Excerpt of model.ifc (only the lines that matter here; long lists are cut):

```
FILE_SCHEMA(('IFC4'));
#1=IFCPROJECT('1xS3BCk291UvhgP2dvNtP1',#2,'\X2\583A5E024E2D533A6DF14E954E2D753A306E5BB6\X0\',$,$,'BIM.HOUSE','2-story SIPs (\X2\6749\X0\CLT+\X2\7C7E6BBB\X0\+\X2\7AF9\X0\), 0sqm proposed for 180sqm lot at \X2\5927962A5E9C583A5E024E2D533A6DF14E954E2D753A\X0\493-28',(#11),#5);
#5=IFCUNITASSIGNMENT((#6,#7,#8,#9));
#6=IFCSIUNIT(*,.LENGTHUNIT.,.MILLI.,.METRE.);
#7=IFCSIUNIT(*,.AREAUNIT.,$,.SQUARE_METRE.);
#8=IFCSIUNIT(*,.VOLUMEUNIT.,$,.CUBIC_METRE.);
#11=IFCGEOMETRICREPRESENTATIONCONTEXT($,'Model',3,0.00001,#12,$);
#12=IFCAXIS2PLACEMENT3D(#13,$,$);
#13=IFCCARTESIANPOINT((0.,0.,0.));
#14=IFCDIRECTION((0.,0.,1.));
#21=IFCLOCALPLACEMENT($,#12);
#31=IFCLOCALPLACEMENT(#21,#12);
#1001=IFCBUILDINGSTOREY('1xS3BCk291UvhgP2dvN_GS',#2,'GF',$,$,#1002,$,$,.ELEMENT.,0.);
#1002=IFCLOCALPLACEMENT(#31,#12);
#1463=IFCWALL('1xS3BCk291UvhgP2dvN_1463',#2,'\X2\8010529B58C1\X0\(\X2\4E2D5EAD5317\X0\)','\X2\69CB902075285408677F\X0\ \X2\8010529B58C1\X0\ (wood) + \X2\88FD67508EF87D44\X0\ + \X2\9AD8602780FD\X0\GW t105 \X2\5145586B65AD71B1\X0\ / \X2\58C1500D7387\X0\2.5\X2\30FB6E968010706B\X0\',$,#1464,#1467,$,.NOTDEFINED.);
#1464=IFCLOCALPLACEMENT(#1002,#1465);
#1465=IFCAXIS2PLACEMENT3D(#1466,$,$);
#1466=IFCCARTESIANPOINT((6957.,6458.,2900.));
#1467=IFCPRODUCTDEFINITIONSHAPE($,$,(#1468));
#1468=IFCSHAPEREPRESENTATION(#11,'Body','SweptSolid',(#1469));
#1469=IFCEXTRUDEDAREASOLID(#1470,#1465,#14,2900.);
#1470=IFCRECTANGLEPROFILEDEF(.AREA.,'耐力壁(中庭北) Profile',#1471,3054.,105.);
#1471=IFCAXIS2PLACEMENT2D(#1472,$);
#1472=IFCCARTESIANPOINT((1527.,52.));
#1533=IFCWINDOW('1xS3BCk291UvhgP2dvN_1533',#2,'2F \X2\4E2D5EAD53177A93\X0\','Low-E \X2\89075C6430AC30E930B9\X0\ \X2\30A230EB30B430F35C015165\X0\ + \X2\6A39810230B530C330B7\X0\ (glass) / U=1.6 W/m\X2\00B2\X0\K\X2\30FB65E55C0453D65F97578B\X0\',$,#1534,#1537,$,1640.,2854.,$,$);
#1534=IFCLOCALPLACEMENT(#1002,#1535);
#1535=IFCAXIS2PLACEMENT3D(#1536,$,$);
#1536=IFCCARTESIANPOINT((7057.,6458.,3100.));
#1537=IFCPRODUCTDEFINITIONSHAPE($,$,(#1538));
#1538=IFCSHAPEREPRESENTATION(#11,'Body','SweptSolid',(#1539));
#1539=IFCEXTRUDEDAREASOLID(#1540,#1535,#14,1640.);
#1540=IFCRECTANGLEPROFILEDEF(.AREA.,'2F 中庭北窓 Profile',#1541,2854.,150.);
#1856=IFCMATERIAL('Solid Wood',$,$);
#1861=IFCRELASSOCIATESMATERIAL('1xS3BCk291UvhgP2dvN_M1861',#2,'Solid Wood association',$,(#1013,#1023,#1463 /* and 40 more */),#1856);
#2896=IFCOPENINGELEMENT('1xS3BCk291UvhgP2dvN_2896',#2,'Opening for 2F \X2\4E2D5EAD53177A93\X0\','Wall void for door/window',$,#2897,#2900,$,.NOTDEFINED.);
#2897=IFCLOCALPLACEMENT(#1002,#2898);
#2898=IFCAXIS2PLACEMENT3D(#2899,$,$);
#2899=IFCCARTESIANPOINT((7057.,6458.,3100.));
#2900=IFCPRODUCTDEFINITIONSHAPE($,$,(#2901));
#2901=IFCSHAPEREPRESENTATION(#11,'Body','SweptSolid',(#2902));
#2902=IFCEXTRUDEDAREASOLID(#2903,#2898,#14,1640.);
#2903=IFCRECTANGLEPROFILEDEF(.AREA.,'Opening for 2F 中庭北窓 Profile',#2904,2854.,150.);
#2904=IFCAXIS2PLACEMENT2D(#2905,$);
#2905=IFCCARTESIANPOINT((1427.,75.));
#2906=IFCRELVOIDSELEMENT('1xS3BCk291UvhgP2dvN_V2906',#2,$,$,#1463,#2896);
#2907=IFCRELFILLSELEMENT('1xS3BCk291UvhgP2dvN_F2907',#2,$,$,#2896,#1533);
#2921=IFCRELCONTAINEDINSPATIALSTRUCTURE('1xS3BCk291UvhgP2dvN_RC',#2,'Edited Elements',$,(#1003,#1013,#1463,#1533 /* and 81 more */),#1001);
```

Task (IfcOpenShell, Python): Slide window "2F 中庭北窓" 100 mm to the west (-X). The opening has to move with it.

```python
import ifcopenshell
import ifcopenshell.api.geometry
import ifcopenshell.util.placement
import ifcopenshell.util.unit

model = ifcopenshell.open("model.ifc")
unit_scale = ifcopenshell.util.unit.calculate_unit_scale(model)

window = model.by_id(1533)
opening = window.FillsVoids[0].RelatingOpeningElement
wall = opening.VoidsElements[0].RelatingBuildingElement

wall_matrix = ifcopenshell.util.placement.get_local_placement(wall.ObjectPlacement)
shift = wall_matrix[:3, 0] * -0.1 / unit_scale
before = ifcopenshell.util.placement.get_local_placement(window.ObjectPlacement)[:3, 3].copy()

# The window is not placed relative to its opening, so move both.
for product in (opening, window):
    matrix = ifcopenshell.util.placement.get_local_placement(product.ObjectPlacement)
    matrix[:3, 3] += shift
    ifcopenshell.api.geometry.edit_object_placement(model, product=product, matrix=matrix, is_si=False)

after = ifcopenshell.util.placement.get_local_placement(window.ObjectPlacement)[:3, 3]
print("window moved by", (after - before).round(3) + 0.0)

model.write("model_edited.ifc")
```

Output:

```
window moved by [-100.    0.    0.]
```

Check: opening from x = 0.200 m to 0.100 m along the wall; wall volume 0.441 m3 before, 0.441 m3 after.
